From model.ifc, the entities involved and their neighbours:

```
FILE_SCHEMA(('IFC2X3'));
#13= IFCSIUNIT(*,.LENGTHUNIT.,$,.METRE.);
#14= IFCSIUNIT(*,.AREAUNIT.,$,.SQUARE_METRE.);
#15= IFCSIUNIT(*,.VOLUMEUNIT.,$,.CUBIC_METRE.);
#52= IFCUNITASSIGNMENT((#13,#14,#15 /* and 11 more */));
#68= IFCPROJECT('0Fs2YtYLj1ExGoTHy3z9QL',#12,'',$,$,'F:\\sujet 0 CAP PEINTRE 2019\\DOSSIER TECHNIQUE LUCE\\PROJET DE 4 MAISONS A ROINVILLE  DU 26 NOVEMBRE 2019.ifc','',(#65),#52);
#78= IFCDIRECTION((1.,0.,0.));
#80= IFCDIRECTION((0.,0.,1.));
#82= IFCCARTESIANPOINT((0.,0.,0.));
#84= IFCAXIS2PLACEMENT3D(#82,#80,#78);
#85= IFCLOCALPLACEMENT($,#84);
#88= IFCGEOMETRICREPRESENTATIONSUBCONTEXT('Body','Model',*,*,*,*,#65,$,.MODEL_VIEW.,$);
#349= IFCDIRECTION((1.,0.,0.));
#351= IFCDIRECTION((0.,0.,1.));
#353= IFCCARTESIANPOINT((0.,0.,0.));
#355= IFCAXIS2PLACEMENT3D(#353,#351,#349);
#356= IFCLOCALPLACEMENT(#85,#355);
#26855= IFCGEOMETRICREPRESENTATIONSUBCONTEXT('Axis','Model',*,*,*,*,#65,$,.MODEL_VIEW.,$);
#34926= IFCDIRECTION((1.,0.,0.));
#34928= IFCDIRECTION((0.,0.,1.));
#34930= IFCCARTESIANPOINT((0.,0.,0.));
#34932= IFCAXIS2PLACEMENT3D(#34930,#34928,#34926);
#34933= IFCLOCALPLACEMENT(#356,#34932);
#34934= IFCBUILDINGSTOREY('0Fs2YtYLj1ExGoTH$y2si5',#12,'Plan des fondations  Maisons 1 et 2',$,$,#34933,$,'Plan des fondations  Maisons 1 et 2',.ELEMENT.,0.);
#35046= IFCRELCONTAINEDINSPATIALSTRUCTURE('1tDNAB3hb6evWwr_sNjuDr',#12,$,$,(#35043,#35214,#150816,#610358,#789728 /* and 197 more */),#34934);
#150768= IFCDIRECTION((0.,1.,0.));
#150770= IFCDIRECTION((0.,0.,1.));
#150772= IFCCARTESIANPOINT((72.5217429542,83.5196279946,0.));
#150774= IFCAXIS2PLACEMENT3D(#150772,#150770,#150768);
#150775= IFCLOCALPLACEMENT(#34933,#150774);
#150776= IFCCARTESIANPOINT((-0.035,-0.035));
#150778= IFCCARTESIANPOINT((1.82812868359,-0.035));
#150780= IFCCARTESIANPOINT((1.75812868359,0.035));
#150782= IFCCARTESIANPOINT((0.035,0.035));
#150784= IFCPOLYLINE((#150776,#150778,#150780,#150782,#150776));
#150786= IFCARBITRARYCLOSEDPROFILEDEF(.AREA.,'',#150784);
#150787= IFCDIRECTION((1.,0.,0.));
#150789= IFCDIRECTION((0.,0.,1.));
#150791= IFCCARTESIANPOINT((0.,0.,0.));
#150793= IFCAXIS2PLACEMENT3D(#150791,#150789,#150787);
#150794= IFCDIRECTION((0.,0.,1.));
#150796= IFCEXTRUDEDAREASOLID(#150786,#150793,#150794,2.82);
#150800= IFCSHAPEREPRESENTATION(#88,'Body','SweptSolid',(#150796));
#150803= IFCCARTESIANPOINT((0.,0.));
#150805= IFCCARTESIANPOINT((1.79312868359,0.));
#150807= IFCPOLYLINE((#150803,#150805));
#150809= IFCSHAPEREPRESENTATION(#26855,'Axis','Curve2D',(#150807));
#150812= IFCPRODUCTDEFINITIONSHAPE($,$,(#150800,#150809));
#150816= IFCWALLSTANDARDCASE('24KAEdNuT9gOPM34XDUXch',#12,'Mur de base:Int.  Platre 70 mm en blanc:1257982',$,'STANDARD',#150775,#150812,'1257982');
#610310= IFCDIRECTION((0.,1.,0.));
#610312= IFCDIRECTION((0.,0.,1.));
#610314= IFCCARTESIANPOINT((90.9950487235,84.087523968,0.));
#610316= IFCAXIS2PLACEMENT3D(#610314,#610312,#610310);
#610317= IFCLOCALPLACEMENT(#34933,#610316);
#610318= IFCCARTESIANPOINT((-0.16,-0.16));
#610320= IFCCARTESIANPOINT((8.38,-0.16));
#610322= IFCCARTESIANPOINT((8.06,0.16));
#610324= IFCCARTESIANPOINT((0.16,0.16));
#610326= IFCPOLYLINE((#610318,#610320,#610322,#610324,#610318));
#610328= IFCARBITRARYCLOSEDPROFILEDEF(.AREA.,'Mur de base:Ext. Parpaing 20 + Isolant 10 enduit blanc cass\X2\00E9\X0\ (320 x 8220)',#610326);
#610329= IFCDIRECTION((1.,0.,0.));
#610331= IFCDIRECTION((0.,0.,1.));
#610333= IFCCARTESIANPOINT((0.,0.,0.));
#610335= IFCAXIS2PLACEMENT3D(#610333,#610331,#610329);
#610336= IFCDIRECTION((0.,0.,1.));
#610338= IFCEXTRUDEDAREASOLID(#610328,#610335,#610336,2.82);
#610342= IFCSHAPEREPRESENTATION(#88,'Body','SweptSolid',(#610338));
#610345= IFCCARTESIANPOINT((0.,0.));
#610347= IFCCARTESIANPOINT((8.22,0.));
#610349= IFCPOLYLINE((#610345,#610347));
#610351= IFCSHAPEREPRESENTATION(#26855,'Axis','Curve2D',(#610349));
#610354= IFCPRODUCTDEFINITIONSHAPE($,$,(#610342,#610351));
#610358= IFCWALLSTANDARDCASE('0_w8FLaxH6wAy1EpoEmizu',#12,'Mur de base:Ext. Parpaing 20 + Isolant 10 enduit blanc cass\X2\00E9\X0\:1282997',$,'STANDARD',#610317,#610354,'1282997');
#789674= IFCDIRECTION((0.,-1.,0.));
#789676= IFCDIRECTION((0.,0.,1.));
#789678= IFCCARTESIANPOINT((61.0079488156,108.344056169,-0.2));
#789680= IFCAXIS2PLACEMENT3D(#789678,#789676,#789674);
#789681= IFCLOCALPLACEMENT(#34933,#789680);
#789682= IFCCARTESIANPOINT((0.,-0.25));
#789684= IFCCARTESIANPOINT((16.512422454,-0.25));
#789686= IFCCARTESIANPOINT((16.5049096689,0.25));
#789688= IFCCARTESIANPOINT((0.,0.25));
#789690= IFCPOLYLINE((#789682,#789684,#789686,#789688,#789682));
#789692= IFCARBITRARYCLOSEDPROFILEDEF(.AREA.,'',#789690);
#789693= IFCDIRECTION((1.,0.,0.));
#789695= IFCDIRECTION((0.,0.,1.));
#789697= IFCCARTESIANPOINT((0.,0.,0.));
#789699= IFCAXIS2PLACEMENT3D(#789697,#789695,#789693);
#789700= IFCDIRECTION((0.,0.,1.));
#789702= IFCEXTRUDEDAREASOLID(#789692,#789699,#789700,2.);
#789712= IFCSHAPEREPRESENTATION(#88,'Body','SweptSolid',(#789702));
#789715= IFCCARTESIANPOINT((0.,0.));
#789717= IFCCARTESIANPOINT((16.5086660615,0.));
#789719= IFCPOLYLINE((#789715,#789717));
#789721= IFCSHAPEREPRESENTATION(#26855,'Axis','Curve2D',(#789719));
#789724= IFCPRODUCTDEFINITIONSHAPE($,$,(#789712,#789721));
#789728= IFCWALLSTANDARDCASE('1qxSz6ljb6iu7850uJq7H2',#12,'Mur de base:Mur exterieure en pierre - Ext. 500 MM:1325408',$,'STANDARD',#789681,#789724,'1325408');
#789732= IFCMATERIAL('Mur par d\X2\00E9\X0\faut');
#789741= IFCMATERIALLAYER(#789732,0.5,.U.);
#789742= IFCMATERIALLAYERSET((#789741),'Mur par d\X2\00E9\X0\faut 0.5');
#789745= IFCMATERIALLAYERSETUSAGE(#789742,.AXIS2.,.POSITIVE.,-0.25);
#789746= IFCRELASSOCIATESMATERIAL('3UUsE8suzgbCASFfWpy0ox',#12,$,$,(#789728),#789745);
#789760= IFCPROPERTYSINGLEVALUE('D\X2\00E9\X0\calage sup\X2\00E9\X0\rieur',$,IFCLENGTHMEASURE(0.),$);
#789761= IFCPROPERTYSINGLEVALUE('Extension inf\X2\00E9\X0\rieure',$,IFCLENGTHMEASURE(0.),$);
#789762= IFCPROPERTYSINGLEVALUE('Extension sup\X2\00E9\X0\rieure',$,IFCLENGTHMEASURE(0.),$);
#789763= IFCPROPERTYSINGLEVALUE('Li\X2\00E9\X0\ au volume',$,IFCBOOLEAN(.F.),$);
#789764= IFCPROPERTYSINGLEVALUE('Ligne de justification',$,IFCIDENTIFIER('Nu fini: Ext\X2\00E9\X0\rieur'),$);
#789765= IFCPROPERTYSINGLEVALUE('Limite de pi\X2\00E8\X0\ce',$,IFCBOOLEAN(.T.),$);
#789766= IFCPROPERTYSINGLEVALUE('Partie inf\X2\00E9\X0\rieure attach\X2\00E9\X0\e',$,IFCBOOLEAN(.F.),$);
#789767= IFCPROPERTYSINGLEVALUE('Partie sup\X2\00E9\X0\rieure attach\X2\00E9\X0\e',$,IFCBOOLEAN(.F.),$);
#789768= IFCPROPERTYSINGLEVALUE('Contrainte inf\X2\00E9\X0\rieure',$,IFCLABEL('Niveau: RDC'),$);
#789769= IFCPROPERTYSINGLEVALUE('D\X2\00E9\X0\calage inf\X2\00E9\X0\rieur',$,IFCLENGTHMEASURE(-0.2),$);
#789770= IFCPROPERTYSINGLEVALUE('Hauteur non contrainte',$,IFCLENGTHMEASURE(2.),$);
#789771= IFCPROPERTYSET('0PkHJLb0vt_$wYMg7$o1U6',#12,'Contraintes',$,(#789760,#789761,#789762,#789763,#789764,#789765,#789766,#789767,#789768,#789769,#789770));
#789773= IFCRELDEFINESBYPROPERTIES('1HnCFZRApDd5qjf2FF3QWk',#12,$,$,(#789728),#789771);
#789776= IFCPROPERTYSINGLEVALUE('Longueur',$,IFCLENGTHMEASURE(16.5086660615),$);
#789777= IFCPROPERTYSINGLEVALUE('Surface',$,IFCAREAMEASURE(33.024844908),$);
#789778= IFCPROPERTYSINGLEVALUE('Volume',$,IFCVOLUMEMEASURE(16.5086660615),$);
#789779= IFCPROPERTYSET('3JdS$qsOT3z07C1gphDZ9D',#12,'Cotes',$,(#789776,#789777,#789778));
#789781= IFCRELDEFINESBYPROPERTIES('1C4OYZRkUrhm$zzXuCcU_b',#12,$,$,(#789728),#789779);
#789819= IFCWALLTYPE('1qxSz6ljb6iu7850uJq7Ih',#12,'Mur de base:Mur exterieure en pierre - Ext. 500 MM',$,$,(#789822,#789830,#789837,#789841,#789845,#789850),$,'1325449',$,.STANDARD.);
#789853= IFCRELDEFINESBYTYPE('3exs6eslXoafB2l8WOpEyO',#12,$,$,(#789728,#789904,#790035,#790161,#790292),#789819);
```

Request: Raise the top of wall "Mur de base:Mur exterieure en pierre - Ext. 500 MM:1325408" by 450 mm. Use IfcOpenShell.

```python
import ifcopenshell
import ifcopenshell.api.pset
import ifcopenshell.geom
import ifcopenshell.util.element
import ifcopenshell.util.representation
import ifcopenshell.util.shape
import ifcopenshell.util.unit

model = ifcopenshell.open("model.ifc")
unit_scale = ifcopenshell.util.unit.calculate_unit_scale(model)
area_scale = ifcopenshell.util.unit.calculate_unit_scale(model, "AREAUNIT")
volume_scale = ifcopenshell.util.unit.calculate_unit_scale(model, "VOLUMEUNIT")
settings = ifcopenshell.geom.settings()


def volume(element):
    """Net volume in cubic metres, openings subtracted."""
    shape = ifcopenshell.geom.create_shape(settings, element)
    return ifcopenshell.util.shape.get_volume(shape.geometry)


wall = model.by_guid("1qxSz6ljb6iu7850uJq7H2")
before = volume(wall)

body = ifcopenshell.util.representation.get_representation(wall, "Model", "Body")
solid = body.Items[0]
old_height = solid.Depth
solid.Depth += 0.45 / unit_scale
after = volume(wall)
thickness = 0.5  # wall thickness in metres

# Update the stored height, areas and volumes.
pset = model.by_id(ifcopenshell.util.element.get_pset(wall, "Contraintes", should_inherit=False)["id"])
ifcopenshell.api.pset.edit_pset(model, pset=pset, properties={
    "Hauteur non contrainte": model.create_entity("IfcLengthMeasure", solid.Depth),
})
pset = model.by_id(ifcopenshell.util.element.get_pset(wall, "Cotes", should_inherit=False)["id"])
ifcopenshell.api.pset.edit_pset(model, pset=pset, properties={
    "Surface": model.create_entity("IfcAreaMeasure", after / thickness / area_scale),
    "Volume": model.create_entity("IfcVolumeMeasure", after / volume_scale),
})

print(f"height {old_height:g} -> {solid.Depth:g}, volume {before:.3f} -> {after:.3f} m3")

model.write("model_updated.ifc")
```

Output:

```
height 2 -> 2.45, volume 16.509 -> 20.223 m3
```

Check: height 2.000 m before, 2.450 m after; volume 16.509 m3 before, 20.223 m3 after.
